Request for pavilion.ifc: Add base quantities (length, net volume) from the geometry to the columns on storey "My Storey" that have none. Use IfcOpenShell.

First a look at what the model holds.

```python
import ifcopenshell
import ifcopenshell.util.element
import ifcopenshell.util.unit

model = ifcopenshell.open("pavilion.ifc")
print(model.schema)
for unit_type in ("LENGTHUNIT", "AREAUNIT", "VOLUMEUNIT"):
    print(unit_type, ifcopenshell.util.unit.calculate_unit_scale(model, unit_type))
storey = next(s for s in model.by_type("IfcBuildingStorey") if s.Name == "My Storey")
columns = [e for e in ifcopenshell.util.element.get_decomposition(storey) if e.is_a("IfcColumn")]
for e in sorted(columns, key=lambda e: e.id()):
    print(e.id(), e.is_a(), e.Name, list(ifcopenshell.util.element.get_psets(e, qtos_only=True)), sep=" | ")
```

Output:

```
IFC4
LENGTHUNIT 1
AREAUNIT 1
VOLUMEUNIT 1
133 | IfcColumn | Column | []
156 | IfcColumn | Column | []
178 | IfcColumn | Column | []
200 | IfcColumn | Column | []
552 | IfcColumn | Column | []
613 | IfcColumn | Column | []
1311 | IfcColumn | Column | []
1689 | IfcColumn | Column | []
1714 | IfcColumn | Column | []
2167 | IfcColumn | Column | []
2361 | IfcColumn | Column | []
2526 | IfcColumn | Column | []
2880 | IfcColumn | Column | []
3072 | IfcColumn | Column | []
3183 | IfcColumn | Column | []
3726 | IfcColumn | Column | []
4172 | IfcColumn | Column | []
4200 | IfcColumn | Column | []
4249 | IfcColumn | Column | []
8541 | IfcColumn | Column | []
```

```python
import ifcopenshell
import ifcopenshell.api.pset
import ifcopenshell.geom
import ifcopenshell.util.element
import ifcopenshell.util.shape
import ifcopenshell.util.unit

model = ifcopenshell.open("pavilion.ifc")
unit_scale = ifcopenshell.util.unit.calculate_unit_scale(model)
volume_scale = ifcopenshell.util.unit.calculate_unit_scale(model, "VOLUMEUNIT")
settings = ifcopenshell.geom.settings()

storey = next(s for s in model.by_type("IfcBuildingStorey") if s.Name == "My Storey")
columns = [e for e in ifcopenshell.util.element.get_decomposition(storey) if e.is_a("IfcColumn")]

for e in sorted(columns, key=lambda e: e.id()):
    if ifcopenshell.util.element.get_psets(e, qtos_only=True, should_inherit=False):
        continue
    # Geometry comes back in metres, in the element's own axes.
    shape = ifcopenshell.geom.create_shape(settings, e)
    values = {
        "Length": ifcopenshell.util.shape.get_z(shape.geometry) / unit_scale,
        "NetVolume": ifcopenshell.util.shape.get_volume(shape.geometry) / volume_scale,
    }
    qto = ifcopenshell.api.pset.add_qto(model, product=e, name="Qto_ColumnBaseQuantities")
    ifcopenshell.api.pset.edit_qto(model, qto=qto, properties=values)
    print(e.id(), {k: round(v, 3) for k, v in values.items()})

model.write("pavilion-out.ifc")
```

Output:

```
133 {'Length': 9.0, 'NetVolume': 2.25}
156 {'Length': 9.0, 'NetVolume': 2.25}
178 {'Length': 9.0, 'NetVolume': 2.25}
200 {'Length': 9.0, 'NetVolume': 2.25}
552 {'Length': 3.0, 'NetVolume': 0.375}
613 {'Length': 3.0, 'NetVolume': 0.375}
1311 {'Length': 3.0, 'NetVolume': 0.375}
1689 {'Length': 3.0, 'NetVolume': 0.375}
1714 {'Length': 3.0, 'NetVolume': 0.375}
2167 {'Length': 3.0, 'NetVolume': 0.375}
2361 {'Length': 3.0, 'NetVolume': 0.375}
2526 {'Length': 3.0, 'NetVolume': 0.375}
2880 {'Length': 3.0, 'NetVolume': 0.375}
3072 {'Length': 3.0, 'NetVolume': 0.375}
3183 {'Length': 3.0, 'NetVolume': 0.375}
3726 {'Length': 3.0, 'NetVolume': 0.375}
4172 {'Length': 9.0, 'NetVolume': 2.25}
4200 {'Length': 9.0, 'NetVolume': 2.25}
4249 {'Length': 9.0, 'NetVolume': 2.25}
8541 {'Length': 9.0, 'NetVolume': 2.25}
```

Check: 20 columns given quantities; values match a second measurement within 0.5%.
